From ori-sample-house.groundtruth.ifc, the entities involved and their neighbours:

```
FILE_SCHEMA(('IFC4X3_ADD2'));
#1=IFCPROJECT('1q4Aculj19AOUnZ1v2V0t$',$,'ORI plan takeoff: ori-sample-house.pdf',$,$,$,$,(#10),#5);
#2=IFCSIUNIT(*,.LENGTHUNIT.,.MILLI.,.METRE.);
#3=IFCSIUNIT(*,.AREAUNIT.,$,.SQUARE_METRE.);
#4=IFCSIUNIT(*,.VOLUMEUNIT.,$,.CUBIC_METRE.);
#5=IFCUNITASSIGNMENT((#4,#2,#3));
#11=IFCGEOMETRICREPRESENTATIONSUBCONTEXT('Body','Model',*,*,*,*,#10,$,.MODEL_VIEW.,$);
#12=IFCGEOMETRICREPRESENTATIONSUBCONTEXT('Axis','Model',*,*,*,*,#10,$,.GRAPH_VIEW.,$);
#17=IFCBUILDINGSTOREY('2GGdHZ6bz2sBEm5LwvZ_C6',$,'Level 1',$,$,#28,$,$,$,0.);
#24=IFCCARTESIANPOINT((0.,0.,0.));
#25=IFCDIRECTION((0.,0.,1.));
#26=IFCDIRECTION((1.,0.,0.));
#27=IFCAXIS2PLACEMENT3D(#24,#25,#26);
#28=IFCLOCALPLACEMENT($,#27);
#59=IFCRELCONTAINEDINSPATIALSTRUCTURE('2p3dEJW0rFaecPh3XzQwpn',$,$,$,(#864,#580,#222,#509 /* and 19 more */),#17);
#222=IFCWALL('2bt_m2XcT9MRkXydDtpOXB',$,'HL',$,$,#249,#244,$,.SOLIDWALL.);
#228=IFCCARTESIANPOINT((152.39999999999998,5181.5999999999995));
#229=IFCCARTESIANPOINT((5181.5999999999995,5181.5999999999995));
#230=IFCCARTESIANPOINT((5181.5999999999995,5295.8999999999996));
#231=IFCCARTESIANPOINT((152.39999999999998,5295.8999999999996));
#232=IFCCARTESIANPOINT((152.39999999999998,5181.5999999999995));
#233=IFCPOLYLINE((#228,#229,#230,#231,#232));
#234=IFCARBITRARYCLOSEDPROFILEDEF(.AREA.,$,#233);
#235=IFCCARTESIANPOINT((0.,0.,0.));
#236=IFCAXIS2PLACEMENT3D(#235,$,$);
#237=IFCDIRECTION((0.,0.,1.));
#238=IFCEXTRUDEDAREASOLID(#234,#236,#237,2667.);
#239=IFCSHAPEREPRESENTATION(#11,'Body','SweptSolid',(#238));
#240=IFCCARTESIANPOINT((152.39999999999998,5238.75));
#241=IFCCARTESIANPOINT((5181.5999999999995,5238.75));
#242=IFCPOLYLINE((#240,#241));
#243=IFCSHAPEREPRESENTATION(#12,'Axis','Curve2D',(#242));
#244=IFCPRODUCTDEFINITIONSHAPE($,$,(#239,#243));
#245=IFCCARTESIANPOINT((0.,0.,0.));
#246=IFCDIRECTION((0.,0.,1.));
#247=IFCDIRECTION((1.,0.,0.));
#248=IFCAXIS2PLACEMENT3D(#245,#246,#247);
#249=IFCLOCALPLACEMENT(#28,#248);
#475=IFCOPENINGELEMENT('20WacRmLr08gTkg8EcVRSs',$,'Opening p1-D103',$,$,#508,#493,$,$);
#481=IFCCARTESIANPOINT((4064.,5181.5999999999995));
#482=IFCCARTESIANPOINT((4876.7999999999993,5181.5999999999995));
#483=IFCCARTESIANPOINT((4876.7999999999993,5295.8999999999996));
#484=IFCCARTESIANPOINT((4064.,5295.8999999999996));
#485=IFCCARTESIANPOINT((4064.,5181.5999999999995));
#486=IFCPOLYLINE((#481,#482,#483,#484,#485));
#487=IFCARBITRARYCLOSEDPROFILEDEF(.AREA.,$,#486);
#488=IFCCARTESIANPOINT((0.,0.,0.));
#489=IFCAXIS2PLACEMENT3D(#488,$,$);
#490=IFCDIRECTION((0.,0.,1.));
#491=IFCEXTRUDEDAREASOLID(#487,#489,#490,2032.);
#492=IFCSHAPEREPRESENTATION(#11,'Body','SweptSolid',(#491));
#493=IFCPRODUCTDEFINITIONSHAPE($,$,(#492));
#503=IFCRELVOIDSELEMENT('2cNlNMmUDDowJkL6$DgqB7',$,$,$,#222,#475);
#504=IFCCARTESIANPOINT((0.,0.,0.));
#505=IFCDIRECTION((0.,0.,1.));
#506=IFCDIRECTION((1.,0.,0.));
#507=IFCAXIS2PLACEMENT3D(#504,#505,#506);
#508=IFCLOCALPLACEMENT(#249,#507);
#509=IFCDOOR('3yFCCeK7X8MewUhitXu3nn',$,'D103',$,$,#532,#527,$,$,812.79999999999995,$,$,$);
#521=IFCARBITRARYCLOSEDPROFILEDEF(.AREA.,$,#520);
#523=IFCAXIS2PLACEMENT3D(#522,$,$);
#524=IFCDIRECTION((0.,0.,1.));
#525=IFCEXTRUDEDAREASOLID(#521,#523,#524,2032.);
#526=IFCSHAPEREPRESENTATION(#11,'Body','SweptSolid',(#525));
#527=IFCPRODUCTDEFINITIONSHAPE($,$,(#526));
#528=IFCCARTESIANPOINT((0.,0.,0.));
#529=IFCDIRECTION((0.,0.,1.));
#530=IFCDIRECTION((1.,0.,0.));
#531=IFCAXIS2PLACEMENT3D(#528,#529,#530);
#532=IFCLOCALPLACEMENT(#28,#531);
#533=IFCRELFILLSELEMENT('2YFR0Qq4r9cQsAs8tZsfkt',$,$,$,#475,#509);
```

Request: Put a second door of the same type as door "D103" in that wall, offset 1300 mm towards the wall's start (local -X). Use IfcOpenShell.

```python
import ifcopenshell
import ifcopenshell.api.feature
import ifcopenshell.api.geometry
import ifcopenshell.api.root
import ifcopenshell.geom
import ifcopenshell.util.element
import ifcopenshell.util.placement
import ifcopenshell.util.shape
import ifcopenshell.util.unit

model = ifcopenshell.open("ori-sample-house.groundtruth.ifc")
unit_scale = ifcopenshell.util.unit.calculate_unit_scale(model)
settings = ifcopenshell.geom.settings()


def volume(element):
    """Net volume in cubic metres, openings subtracted."""
    shape = ifcopenshell.geom.create_shape(settings, element)
    return ifcopenshell.util.shape.get_volume(shape.geometry)


door = model.by_id(509)
opening = door.FillsVoids[0].RelatingOpeningElement
wall = opening.VoidsElements[0].RelatingBuildingElement
before = volume(wall)
shift = ifcopenshell.util.placement.get_local_placement(wall.ObjectPlacement)[:3, 0] * -1.3 / unit_scale

# copy_class copies the void relationship, type, container and properties, but no geometry.
new_opening = ifcopenshell.api.root.copy_class(model, product=opening)
new_opening.Representation = ifcopenshell.util.element.copy_deep(
    model, opening.Representation, exclude=["IfcGeometricRepresentationContext", "IfcRepresentationMap"]
)
new_door = ifcopenshell.api.root.copy_class(model, product=door)
new_door.Representation = ifcopenshell.util.element.copy_deep(
    model, door.Representation, exclude=["IfcGeometricRepresentationContext", "IfcRepresentationMap"]
)
ifcopenshell.api.feature.add_filling(model, opening=new_opening, element=new_door)

for old, new in ((opening, new_opening), (door, new_door)):
    matrix = ifcopenshell.util.placement.get_local_placement(old.ObjectPlacement)
    matrix[:3, 3] += shift
    ifcopenshell.api.geometry.edit_object_placement(model, product=new, matrix=matrix, is_si=False)

after = volume(wall)

print(f"wall volume {before:.3f} -> {after:.3f} m3")

model.write("ori-sample-house.groundtruth_rev.ifc")
```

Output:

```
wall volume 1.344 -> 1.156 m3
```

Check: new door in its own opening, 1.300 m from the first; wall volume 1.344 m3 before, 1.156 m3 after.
